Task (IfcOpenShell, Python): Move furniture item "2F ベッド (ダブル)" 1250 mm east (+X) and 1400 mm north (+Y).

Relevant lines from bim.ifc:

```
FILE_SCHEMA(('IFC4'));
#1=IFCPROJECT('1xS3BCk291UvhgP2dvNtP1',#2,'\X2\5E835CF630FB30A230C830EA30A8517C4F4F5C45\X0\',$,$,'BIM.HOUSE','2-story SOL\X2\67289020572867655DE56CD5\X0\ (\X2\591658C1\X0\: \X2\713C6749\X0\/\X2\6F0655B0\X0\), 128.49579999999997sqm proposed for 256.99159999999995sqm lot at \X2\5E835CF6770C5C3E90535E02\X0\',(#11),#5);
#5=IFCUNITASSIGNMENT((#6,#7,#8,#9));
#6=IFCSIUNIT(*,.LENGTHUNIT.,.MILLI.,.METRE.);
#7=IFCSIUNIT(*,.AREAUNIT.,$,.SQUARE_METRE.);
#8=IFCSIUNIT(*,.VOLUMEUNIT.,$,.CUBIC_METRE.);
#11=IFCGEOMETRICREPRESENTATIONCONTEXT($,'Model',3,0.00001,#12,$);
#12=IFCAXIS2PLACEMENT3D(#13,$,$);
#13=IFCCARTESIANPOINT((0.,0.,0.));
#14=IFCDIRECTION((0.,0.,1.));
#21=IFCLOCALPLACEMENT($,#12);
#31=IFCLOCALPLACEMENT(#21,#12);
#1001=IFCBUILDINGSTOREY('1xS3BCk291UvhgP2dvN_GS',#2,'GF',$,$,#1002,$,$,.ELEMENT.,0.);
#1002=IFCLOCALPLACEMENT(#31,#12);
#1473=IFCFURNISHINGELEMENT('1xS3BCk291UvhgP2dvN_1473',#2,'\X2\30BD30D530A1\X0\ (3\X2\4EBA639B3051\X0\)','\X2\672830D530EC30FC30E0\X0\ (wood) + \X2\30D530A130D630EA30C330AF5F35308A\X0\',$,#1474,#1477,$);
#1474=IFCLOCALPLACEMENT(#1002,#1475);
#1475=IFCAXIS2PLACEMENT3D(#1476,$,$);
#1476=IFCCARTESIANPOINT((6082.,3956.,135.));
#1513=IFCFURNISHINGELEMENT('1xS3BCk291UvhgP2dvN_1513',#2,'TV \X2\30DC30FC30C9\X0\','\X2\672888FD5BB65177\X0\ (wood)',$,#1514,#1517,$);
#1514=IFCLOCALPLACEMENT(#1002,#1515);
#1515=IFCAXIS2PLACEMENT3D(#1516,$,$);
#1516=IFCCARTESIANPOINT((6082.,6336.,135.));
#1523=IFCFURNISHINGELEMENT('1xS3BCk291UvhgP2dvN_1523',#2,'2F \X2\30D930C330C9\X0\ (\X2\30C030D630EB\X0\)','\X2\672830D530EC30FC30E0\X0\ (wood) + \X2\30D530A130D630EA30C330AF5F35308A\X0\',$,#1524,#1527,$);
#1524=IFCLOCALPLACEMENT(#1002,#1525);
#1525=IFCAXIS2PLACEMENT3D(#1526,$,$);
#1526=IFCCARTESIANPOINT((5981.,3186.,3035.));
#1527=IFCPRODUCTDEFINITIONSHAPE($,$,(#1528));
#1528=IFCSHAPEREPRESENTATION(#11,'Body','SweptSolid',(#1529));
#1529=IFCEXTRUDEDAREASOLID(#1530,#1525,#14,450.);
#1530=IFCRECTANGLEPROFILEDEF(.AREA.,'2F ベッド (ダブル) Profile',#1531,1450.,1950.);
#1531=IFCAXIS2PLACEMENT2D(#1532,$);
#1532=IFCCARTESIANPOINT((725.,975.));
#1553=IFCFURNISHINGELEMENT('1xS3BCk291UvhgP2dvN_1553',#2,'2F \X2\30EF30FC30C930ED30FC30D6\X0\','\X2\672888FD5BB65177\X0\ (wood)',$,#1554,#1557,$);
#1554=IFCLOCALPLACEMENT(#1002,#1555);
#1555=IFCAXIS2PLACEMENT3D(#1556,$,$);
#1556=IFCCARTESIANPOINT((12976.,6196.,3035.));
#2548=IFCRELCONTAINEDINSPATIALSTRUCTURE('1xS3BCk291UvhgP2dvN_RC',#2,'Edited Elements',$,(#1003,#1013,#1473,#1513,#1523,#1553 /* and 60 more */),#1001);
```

```python
import ifcopenshell
import ifcopenshell.api.geometry
import ifcopenshell.util.placement

model = ifcopenshell.open("bim.ifc")

item = model.by_id(1523)
matrix = ifcopenshell.util.placement.get_local_placement(item.ObjectPlacement)
matrix[0, 3] += 1250.0
matrix[1, 3] += 1400.0
ifcopenshell.api.geometry.edit_object_placement(model, product=item, matrix=matrix, is_si=False)

print(ifcopenshell.util.placement.get_local_placement(item.ObjectPlacement).round(3) + 0.0)

model.write("bim_rev.ifc")
```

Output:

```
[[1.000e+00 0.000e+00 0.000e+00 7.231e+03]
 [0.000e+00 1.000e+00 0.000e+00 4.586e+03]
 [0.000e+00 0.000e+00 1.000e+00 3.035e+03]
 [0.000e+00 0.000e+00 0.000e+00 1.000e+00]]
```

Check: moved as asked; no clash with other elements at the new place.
